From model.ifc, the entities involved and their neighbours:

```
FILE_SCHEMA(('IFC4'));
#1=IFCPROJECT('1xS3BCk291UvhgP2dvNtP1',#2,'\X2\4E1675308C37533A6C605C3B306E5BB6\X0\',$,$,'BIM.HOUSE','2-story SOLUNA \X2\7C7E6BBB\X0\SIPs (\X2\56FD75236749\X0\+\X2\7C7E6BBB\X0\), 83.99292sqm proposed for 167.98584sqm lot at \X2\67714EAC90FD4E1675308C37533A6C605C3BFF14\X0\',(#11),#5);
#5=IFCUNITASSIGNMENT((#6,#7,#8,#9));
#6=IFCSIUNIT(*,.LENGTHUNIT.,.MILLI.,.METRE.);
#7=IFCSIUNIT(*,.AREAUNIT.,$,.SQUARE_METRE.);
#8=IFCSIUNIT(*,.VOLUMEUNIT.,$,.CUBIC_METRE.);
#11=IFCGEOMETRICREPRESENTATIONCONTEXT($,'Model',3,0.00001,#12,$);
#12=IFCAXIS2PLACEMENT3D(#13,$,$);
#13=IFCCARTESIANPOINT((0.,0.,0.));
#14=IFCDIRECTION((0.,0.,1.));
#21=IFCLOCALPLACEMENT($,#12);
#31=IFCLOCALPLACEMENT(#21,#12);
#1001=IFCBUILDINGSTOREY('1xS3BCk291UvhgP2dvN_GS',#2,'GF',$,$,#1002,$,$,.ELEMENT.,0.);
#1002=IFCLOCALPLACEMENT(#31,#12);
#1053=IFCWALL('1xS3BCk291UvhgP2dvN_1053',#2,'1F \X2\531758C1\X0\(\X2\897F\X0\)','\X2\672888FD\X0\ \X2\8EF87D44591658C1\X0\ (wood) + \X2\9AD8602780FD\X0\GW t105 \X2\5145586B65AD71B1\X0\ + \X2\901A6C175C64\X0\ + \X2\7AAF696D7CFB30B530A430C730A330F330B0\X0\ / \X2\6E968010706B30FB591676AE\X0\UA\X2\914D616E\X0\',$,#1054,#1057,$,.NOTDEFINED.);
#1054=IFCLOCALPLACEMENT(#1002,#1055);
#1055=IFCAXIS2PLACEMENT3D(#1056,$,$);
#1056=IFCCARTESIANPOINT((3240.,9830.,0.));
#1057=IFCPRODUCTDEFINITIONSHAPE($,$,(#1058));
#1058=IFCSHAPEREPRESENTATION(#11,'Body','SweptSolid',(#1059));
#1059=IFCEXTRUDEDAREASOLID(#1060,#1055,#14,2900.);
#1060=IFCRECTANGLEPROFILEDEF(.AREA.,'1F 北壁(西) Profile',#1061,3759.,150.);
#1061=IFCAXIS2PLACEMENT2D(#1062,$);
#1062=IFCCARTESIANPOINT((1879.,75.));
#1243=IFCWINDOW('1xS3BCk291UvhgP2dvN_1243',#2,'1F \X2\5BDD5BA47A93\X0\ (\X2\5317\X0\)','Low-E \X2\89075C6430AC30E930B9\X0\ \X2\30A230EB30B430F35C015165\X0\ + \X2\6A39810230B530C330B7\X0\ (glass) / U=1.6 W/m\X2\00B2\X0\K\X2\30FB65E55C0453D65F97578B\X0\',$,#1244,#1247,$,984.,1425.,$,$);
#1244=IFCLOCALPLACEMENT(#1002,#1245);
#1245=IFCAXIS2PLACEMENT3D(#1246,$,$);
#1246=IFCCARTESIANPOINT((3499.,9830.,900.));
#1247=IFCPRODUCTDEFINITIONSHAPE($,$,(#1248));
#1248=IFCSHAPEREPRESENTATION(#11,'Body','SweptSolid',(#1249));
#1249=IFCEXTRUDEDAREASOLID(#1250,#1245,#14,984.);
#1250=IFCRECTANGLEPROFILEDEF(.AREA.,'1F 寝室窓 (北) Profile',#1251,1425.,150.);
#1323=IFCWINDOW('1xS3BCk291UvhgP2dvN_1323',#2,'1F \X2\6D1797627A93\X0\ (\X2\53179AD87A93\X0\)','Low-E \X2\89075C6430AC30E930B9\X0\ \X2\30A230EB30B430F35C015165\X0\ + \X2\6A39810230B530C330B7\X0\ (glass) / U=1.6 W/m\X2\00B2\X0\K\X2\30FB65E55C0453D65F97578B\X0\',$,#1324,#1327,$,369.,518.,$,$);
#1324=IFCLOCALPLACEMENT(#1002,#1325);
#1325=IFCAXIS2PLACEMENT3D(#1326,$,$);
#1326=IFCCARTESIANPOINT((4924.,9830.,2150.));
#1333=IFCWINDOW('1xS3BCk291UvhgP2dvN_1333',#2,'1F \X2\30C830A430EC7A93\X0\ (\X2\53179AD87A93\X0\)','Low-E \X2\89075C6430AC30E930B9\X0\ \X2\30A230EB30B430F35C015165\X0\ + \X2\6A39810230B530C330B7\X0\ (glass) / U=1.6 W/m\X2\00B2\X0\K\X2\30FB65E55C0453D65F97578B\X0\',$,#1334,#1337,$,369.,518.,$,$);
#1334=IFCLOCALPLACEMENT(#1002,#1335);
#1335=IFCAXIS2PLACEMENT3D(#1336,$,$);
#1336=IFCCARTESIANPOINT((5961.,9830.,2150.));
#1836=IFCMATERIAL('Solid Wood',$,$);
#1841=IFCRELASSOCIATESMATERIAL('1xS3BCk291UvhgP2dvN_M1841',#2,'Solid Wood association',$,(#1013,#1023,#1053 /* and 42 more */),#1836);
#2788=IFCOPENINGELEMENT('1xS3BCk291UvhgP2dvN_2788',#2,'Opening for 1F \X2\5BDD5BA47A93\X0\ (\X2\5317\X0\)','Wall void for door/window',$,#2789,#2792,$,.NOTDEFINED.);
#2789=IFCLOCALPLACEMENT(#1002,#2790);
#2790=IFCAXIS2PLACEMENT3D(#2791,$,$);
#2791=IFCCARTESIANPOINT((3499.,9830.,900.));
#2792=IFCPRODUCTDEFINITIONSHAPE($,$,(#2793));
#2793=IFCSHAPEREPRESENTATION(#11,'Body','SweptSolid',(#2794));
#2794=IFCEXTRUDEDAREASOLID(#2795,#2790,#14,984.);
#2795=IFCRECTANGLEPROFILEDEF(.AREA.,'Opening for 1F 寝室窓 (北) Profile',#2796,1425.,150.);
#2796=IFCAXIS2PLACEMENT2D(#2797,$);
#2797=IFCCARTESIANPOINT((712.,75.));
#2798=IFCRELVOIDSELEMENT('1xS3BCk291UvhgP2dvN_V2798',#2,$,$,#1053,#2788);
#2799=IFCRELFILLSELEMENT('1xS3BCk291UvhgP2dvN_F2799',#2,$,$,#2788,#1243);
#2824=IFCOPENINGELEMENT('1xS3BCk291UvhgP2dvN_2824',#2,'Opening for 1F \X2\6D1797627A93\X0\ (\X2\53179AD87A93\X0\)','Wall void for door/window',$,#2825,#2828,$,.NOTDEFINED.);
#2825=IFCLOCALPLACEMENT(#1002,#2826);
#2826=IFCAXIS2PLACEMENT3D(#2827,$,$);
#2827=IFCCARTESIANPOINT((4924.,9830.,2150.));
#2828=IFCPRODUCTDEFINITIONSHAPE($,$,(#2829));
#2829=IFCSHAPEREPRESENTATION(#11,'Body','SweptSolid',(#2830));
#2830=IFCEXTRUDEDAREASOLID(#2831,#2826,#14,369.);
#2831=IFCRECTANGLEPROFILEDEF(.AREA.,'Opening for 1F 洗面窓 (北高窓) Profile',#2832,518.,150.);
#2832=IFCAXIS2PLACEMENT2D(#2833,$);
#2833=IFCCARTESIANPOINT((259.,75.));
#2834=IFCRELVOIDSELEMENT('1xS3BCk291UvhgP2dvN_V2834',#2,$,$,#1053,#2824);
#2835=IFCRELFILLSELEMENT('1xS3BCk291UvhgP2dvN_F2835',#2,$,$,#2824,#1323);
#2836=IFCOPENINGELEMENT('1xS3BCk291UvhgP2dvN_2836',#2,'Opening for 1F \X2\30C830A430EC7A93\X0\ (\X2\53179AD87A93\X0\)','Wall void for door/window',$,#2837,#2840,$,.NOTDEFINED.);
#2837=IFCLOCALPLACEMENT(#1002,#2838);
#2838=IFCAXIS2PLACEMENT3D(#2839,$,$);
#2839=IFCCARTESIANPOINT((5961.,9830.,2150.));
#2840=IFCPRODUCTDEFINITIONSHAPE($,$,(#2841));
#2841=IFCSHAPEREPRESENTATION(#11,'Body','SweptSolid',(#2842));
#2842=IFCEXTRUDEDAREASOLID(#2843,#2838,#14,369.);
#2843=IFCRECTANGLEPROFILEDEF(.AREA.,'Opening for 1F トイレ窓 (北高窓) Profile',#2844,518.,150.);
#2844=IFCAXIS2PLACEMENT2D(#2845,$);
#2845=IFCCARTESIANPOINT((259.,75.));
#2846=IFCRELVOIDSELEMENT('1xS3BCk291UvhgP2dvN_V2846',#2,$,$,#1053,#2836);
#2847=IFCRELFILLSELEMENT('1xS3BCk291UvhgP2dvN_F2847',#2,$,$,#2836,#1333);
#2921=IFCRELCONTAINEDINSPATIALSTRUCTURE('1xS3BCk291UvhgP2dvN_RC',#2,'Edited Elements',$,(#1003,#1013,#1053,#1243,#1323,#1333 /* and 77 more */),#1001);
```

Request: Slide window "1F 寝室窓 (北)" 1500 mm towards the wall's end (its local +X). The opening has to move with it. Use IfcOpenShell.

```python
import ifcopenshell
import ifcopenshell.api.geometry
import ifcopenshell.util.placement

model = ifcopenshell.open("model.ifc")

window = model.by_id(1243)
opening = window.FillsVoids[0].RelatingOpeningElement
wall = opening.VoidsElements[0].RelatingBuildingElement

wall_matrix = ifcopenshell.util.placement.get_local_placement(wall.ObjectPlacement)
shift = wall_matrix[:3, 0] * 1500.0
before = ifcopenshell.util.placement.get_local_placement(window.ObjectPlacement)[:3, 3].copy()

# The window is not placed relative to its opening, so move both.
for product in (opening, window):
    matrix = ifcopenshell.util.placement.get_local_placement(product.ObjectPlacement)
    matrix[:3, 3] += shift
    ifcopenshell.api.geometry.edit_object_placement(model, product=product, matrix=matrix, is_si=False)

after = ifcopenshell.util.placement.get_local_placement(window.ObjectPlacement)[:3, 3]
print("window moved by", (after - before).round(3) + 0.0)

model.write("model_updated.ifc")
```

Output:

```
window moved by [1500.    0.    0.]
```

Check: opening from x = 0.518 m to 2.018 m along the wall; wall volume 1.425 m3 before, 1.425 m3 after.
